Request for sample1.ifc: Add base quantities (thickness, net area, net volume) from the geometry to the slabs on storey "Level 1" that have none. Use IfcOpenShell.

First a look at what the model holds.

```python
import ifcopenshell
import ifcopenshell.util.element
import ifcopenshell.util.unit

model = ifcopenshell.open("sample1.ifc")
print(model.schema)
for unit_type in ("LENGTHUNIT", "AREAUNIT", "VOLUMEUNIT"):
    print(unit_type, ifcopenshell.util.unit.calculate_unit_scale(model, unit_type))
storey = next(s for s in model.by_type("IfcBuildingStorey") if s.Name == "Level 1")
slabs = [e for e in ifcopenshell.util.element.get_decomposition(storey) if e.is_a("IfcSlab")]
for e in sorted(slabs, key=lambda e: e.id()):
    print(e.id(), e.is_a(), e.Name, list(ifcopenshell.util.element.get_psets(e, qtos_only=True)), sep=" | ")
```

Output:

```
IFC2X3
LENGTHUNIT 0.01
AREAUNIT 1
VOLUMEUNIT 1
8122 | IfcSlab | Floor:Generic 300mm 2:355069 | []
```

```python
import ifcopenshell
import ifcopenshell.api.pset
import ifcopenshell.geom
import ifcopenshell.util.element
import ifcopenshell.util.shape
import ifcopenshell.util.unit

model = ifcopenshell.open("sample1.ifc")
unit_scale = ifcopenshell.util.unit.calculate_unit_scale(model)
area_scale = ifcopenshell.util.unit.calculate_unit_scale(model, "AREAUNIT")
volume_scale = ifcopenshell.util.unit.calculate_unit_scale(model, "VOLUMEUNIT")
settings = ifcopenshell.geom.settings()

storey = next(s for s in model.by_type("IfcBuildingStorey") if s.Name == "Level 1")
slabs = [e for e in ifcopenshell.util.element.get_decomposition(storey) if e.is_a("IfcSlab")]

for e in sorted(slabs, key=lambda e: e.id()):
    if ifcopenshell.util.element.get_psets(e, qtos_only=True, should_inherit=False):
        continue
    # Geometry comes back in metres, in the element's own axes.
    shape = ifcopenshell.geom.create_shape(settings, e)
    values = {
        "Width": ifcopenshell.util.shape.get_z(shape.geometry) / unit_scale,
        "NetArea": ifcopenshell.util.shape.get_footprint_area(shape.geometry) / area_scale,
        "NetVolume": ifcopenshell.util.shape.get_volume(shape.geometry) / volume_scale,
    }
    qto = ifcopenshell.api.pset.add_qto(model, product=e, name="BaseQuantities")
    ifcopenshell.api.pset.edit_qto(model, qto=qto, properties=values)
    print(e.id(), {k: round(v, 3) for k, v in values.items()})

model.write("sample1_updated.ifc")
```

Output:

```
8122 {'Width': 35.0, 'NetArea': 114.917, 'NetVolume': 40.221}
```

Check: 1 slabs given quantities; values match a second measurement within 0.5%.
